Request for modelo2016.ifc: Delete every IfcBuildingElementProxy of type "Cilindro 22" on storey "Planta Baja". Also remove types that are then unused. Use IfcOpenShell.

First a look at what the model holds.

```python
import ifcopenshell
import ifcopenshell.util.element

model = ifcopenshell.open("modelo2016.ifc")
print(model.schema)
storey = next(s for s in model.by_type("IfcBuildingStorey") if s.Name == "Planta Baja")
proxies = [e for e in ifcopenshell.util.element.get_decomposition(storey) if e.is_a("IfcBuildingElementProxy")]
seen = {}
for e in proxies:
    element_type = ifcopenshell.util.element.get_type(e)
    name = element_type.Name if element_type not in (None, e) else None
    seen[name] = seen.get(name, 0) + 1
for name, count in sorted(seen.items(), key=str):
    print(count, "x", name)
```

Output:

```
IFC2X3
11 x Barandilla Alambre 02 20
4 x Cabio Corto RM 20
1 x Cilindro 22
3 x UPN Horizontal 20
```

```python
import ifcopenshell
import ifcopenshell.api.root
import ifcopenshell.util.element

model = ifcopenshell.open("modelo2016.ifc")

storey = next(s for s in model.by_type("IfcBuildingStorey") if s.Name == "Planta Baja")
proxies = [e for e in ifcopenshell.util.element.get_decomposition(storey) if e.is_a("IfcBuildingElementProxy")]
targets = [e for e in proxies if (t := ifcopenshell.util.element.get_type(e)) not in (None, e) and t.Name == "Cilindro 22"]
types = {ifcopenshell.util.element.get_type(e) for e in targets} - {None, *targets}

for e in targets:
    ifcopenshell.api.root.remove_product(model, product=e)
print(len(targets), "removed")

unused = [t for t in types if not ifcopenshell.util.element.get_types(t)]
for t in unused:
    ifcopenshell.api.root.remove_product(model, product=t)
print(len(unused), "unused types removed")

model.write("modelo2016_updated.ifc")
```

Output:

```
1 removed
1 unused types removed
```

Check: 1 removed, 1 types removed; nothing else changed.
